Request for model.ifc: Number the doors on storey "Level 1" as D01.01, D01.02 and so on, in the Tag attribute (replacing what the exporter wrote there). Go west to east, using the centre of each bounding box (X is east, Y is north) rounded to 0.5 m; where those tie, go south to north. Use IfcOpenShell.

First a look at what the model holds.

```python
import ifcopenshell
import ifcopenshell.util.element
import ifcopenshell.util.placement

model = ifcopenshell.open("model.ifc")
print(model.schema)
storey = next(s for s in model.by_type("IfcBuildingStorey") if s.Name == "Level 1")
doors = [e for e in ifcopenshell.util.element.get_decomposition(storey) if e.is_a("IfcDoor")]
for e in sorted(doors, key=lambda e: e.id()):
    origin = ifcopenshell.util.placement.get_local_placement(e.ObjectPlacement)[:3, 3]
    print(e.id(), e.Tag, e.Name, origin.round(2) + 0.0, sep=" | ")
```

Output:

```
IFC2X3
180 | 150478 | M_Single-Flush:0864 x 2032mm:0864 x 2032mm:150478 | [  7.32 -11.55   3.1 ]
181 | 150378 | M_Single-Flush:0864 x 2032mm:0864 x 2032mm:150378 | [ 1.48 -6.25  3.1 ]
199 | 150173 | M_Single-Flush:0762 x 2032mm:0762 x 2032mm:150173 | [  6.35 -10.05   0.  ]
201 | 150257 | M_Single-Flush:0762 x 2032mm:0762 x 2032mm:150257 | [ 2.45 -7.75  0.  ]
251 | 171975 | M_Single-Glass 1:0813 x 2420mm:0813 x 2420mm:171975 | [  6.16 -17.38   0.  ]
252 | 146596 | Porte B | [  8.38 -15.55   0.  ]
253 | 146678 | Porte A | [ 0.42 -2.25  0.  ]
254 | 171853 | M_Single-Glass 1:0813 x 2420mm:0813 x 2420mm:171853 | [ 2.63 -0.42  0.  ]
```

```python
import ifcopenshell
import ifcopenshell.geom
import ifcopenshell.util.element
import ifcopenshell.util.shape

model = ifcopenshell.open("model.ifc")
settings = ifcopenshell.geom.settings()
settings.set("use-world-coords", True)


def centre(element):
    shape = ifcopenshell.geom.create_shape(settings, element)
    return ifcopenshell.util.shape.get_bbox_centroid(shape.geometry)


storey = next(s for s in model.by_type("IfcBuildingStorey") if s.Name == "Level 1")
doors = [e for e in ifcopenshell.util.element.get_decomposition(storey) if e.is_a("IfcDoor")]

# Insertion points can sit at a corner or the storey origin, so sort by the geometry (in metres).
centres = {e: centre(e) for e in doors}
doors.sort(key=lambda e: (round(centres[e][0] / 0.5), centres[e][1]))

for i, e in enumerate(doors, start=1):
    number = f"D01.{i:02d}"
    e.Tag = number
    print(e.id(), number)

model.write("model_rev.ifc")
```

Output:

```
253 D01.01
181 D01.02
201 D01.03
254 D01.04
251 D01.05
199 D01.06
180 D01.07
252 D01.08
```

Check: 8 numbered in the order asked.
